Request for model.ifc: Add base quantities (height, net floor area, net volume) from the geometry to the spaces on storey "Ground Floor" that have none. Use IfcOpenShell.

First a look at what the model holds.

```python
import ifcopenshell
import ifcopenshell.util.element
import ifcopenshell.util.unit

model = ifcopenshell.open("model.ifc")
print(model.schema)
for unit_type in ("LENGTHUNIT", "AREAUNIT", "VOLUMEUNIT"):
    print(unit_type, ifcopenshell.util.unit.calculate_unit_scale(model, unit_type))
storey = next(s for s in model.by_type("IfcBuildingStorey") if s.Name == "Ground Floor")
spaces = [e for e in ifcopenshell.util.element.get_decomposition(storey) if e.is_a("IfcSpace")]
for e in sorted(spaces, key=lambda e: e.id()):
    print(e.id(), e.is_a(), e.Name, list(ifcopenshell.util.element.get_psets(e, qtos_only=True)), sep=" | ")
```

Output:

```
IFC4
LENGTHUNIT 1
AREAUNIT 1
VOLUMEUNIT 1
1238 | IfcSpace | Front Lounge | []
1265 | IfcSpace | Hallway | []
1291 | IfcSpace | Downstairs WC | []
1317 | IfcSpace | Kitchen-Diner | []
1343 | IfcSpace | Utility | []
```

```python
import ifcopenshell
import ifcopenshell.api.pset
import ifcopenshell.geom
import ifcopenshell.util.element
import ifcopenshell.util.shape
import ifcopenshell.util.unit

model = ifcopenshell.open("model.ifc")
unit_scale = ifcopenshell.util.unit.calculate_unit_scale(model)
area_scale = ifcopenshell.util.unit.calculate_unit_scale(model, "AREAUNIT")
volume_scale = ifcopenshell.util.unit.calculate_unit_scale(model, "VOLUMEUNIT")
settings = ifcopenshell.geom.settings()

storey = next(s for s in model.by_type("IfcBuildingStorey") if s.Name == "Ground Floor")
spaces = [e for e in ifcopenshell.util.element.get_decomposition(storey) if e.is_a("IfcSpace")]

for e in sorted(spaces, key=lambda e: e.id()):
    if ifcopenshell.util.element.get_psets(e, qtos_only=True, should_inherit=False):
        continue
    # Geometry comes back in metres, in the element's own axes.
    shape = ifcopenshell.geom.create_shape(settings, e)
    values = {
        "Height": ifcopenshell.util.shape.get_z(shape.geometry) / unit_scale,
        "NetFloorArea": ifcopenshell.util.shape.get_footprint_area(shape.geometry) / area_scale,
        "NetVolume": ifcopenshell.util.shape.get_volume(shape.geometry) / volume_scale,
    }
    qto = ifcopenshell.api.pset.add_qto(model, product=e, name="Qto_SpaceBaseQuantities")
    ifcopenshell.api.pset.edit_qto(model, qto=qto, properties=values)
    print(e.id(), {k: round(v, 3) for k, v in values.items()})

model.write("model_updated.ifc")
```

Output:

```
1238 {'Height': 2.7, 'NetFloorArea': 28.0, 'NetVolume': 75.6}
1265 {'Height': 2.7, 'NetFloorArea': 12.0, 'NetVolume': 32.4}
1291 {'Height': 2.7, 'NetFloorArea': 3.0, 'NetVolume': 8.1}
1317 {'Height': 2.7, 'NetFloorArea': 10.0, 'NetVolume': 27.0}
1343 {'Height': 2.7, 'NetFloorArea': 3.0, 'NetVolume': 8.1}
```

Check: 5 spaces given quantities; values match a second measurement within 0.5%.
